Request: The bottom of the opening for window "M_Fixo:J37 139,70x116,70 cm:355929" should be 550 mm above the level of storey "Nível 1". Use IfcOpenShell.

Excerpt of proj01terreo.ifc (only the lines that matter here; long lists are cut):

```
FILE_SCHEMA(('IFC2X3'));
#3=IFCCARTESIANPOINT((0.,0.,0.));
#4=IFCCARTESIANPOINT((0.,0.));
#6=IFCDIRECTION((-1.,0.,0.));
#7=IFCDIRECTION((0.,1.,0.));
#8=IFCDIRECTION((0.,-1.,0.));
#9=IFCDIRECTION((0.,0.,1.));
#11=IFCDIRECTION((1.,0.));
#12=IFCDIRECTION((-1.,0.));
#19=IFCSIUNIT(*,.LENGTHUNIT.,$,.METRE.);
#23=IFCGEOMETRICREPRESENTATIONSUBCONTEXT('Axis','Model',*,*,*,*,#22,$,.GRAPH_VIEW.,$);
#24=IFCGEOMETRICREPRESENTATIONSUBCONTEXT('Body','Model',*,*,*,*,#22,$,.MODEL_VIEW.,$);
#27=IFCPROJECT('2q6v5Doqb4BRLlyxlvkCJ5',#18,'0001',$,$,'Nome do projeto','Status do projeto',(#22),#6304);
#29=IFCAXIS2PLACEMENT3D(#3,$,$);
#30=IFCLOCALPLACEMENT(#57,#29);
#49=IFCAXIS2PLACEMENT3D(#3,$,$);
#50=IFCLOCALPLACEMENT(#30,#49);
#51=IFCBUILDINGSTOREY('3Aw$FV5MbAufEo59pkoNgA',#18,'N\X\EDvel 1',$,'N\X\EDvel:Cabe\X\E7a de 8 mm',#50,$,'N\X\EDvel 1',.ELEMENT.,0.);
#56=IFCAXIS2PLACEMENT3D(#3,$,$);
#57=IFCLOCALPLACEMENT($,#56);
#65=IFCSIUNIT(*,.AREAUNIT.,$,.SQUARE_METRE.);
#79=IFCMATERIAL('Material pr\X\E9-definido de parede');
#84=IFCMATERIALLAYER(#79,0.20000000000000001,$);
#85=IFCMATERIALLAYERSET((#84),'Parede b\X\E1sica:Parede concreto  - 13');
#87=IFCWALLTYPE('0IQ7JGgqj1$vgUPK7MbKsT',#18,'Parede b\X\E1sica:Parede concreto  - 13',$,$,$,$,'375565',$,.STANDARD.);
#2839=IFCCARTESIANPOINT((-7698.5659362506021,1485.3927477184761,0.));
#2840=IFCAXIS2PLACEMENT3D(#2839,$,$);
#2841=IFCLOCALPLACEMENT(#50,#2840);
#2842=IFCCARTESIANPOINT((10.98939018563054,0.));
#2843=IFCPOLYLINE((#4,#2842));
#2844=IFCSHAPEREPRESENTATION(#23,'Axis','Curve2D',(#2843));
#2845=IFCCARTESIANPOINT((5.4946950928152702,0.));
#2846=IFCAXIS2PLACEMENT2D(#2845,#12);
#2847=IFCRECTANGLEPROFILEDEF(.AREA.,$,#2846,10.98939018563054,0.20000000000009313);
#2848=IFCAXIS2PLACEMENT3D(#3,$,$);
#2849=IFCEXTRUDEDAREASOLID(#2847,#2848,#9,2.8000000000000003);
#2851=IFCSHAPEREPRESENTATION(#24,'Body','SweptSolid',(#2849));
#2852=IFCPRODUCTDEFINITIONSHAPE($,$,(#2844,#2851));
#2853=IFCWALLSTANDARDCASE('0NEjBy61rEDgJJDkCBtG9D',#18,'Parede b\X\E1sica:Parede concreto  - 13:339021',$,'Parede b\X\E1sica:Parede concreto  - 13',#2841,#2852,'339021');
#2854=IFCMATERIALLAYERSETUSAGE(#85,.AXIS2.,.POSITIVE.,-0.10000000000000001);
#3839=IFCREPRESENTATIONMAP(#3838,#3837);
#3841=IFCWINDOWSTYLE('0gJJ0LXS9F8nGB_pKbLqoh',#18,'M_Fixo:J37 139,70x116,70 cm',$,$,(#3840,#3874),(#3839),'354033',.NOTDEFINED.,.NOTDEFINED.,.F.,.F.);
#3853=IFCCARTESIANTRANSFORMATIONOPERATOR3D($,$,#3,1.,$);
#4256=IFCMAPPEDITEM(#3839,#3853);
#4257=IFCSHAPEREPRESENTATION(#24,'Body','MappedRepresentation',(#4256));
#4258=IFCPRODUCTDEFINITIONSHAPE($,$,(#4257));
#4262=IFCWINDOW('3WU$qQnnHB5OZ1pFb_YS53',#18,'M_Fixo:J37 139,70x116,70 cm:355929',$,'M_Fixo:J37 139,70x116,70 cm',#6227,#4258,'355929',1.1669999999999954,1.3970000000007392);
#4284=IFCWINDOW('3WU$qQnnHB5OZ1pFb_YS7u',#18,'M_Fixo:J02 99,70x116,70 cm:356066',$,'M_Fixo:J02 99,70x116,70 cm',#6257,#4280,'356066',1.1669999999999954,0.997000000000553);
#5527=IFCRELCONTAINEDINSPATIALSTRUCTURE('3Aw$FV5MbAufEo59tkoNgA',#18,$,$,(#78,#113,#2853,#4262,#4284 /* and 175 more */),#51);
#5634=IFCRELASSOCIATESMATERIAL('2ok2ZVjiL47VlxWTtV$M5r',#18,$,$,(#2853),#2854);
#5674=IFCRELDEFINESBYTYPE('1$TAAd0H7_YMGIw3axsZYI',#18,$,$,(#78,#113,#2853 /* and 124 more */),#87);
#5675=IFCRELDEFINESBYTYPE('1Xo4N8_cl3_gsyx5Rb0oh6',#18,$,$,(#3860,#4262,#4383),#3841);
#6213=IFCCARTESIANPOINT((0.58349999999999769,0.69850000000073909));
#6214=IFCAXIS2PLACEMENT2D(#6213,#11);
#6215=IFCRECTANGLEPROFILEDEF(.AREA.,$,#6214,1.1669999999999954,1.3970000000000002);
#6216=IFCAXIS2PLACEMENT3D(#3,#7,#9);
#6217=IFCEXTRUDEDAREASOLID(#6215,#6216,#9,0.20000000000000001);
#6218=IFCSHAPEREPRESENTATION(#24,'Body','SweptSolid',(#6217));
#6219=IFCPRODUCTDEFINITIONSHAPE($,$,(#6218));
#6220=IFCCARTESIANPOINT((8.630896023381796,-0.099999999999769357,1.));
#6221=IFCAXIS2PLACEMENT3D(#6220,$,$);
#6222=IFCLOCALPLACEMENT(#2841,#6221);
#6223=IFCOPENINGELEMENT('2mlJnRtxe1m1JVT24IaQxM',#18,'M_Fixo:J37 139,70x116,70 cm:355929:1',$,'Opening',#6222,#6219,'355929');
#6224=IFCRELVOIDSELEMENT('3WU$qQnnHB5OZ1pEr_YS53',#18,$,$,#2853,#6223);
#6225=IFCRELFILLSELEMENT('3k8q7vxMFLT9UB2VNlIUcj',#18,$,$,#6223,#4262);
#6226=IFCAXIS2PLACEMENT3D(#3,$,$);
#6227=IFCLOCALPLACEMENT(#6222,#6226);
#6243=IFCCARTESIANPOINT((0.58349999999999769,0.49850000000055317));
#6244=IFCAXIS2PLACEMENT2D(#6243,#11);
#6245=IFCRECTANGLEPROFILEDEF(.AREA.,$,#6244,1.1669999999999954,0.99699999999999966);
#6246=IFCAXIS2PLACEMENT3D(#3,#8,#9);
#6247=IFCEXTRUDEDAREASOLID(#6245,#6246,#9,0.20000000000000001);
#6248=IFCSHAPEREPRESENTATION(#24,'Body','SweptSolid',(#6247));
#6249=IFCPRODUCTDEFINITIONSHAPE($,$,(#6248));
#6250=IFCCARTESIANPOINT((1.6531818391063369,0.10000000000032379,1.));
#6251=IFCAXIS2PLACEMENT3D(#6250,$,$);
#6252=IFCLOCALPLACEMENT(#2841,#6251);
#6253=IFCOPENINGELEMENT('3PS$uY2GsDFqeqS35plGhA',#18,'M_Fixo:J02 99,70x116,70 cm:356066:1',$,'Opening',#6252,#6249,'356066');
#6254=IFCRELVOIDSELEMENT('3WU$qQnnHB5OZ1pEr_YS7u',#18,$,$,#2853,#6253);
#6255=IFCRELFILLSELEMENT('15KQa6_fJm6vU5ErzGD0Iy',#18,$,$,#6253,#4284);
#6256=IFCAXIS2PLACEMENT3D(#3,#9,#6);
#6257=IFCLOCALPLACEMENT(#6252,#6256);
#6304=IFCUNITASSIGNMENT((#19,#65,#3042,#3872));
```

```python
import numpy as np
import ifcopenshell
import ifcopenshell.api.geometry
import ifcopenshell.geom
import ifcopenshell.util.element
import ifcopenshell.util.placement
import ifcopenshell.util.shape
import ifcopenshell.util.unit

model = ifcopenshell.open("proj01terreo.ifc")
unit_scale = ifcopenshell.util.unit.calculate_unit_scale(model)

window = model.by_guid("3WU$qQnnHB5OZ1pFb_YS53")
opening = window.FillsVoids[0].RelatingOpeningElement
storey = ifcopenshell.util.element.get_container(window, ifc_class="IfcBuildingStorey")
level = ifcopenshell.util.placement.get_local_placement(storey.ObjectPlacement)[2, 3]

# The opening's origin need not be at the sill, so measure its lowest point.
shape = ifcopenshell.geom.create_shape(ifcopenshell.geom.settings(), opening)
bottom = ifcopenshell.util.shape.get_shape_bottom_elevation(shape, shape.geometry) / unit_scale
dz = level + 0.55 - bottom

shift = np.array([0.0, 0.0, dz])
# The window is placed relative to its opening, so it follows when the opening moves.
matrix = ifcopenshell.util.placement.get_local_placement(opening.ObjectPlacement)
matrix[:3, 3] += shift
ifcopenshell.api.geometry.edit_object_placement(
    model, product=opening, matrix=matrix, is_si=False, should_transform_children=True
)

print(f"moved by {dz * unit_scale:+.3f} m")

model.write("proj01terreo_updated.ifc")
```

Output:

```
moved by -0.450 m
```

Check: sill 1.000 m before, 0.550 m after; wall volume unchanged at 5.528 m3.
